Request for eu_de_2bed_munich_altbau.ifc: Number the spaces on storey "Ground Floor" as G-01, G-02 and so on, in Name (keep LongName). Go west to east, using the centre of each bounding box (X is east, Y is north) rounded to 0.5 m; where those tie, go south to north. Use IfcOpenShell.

First a look at what the model holds.

```python
import ifcopenshell
import ifcopenshell.util.element
import ifcopenshell.util.placement

model = ifcopenshell.open("eu_de_2bed_munich_altbau.ifc")
print(model.schema)
storey = next(s for s in model.by_type("IfcBuildingStorey") if s.Name == "Ground Floor")
spaces = [e for e in ifcopenshell.util.element.get_decomposition(storey) if e.is_a("IfcSpace")]
for e in sorted(spaces, key=lambda e: e.id()):
    origin = ifcopenshell.util.placement.get_local_placement(e.ObjectPlacement)[:3, 3]
    print(e.id(), e.Name, e.LongName, origin.round(2) + 0.0, sep=" | ")
```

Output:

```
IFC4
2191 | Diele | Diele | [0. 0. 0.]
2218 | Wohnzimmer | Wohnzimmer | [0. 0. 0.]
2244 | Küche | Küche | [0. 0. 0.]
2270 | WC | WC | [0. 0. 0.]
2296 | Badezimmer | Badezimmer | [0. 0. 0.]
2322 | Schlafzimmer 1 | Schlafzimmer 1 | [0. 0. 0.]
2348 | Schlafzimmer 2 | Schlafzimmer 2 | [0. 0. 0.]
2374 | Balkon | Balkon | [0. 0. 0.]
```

```python
import ifcopenshell
import ifcopenshell.geom
import ifcopenshell.util.element
import ifcopenshell.util.shape

model = ifcopenshell.open("eu_de_2bed_munich_altbau.ifc")
settings = ifcopenshell.geom.settings()
settings.set("use-world-coords", True)


def centre(element):
    shape = ifcopenshell.geom.create_shape(settings, element)
    return ifcopenshell.util.shape.get_bbox_centroid(shape.geometry)


storey = next(s for s in model.by_type("IfcBuildingStorey") if s.Name == "Ground Floor")
spaces = [e for e in ifcopenshell.util.element.get_decomposition(storey) if e.is_a("IfcSpace")]

# Insertion points can sit at a corner or the storey origin, so sort by the geometry (in metres).
centres = {e: centre(e) for e in spaces}
spaces.sort(key=lambda e: (round(centres[e][0] / 0.5), centres[e][1]))

for i, e in enumerate(spaces, start=1):
    number = f"G-{i:02d}"
    e.Name = number
    print(e.id(), number)

model.write("eu_de_2bed_munich_altbau_rev.ifc")
```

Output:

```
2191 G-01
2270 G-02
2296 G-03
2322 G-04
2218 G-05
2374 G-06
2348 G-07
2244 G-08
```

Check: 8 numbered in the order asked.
